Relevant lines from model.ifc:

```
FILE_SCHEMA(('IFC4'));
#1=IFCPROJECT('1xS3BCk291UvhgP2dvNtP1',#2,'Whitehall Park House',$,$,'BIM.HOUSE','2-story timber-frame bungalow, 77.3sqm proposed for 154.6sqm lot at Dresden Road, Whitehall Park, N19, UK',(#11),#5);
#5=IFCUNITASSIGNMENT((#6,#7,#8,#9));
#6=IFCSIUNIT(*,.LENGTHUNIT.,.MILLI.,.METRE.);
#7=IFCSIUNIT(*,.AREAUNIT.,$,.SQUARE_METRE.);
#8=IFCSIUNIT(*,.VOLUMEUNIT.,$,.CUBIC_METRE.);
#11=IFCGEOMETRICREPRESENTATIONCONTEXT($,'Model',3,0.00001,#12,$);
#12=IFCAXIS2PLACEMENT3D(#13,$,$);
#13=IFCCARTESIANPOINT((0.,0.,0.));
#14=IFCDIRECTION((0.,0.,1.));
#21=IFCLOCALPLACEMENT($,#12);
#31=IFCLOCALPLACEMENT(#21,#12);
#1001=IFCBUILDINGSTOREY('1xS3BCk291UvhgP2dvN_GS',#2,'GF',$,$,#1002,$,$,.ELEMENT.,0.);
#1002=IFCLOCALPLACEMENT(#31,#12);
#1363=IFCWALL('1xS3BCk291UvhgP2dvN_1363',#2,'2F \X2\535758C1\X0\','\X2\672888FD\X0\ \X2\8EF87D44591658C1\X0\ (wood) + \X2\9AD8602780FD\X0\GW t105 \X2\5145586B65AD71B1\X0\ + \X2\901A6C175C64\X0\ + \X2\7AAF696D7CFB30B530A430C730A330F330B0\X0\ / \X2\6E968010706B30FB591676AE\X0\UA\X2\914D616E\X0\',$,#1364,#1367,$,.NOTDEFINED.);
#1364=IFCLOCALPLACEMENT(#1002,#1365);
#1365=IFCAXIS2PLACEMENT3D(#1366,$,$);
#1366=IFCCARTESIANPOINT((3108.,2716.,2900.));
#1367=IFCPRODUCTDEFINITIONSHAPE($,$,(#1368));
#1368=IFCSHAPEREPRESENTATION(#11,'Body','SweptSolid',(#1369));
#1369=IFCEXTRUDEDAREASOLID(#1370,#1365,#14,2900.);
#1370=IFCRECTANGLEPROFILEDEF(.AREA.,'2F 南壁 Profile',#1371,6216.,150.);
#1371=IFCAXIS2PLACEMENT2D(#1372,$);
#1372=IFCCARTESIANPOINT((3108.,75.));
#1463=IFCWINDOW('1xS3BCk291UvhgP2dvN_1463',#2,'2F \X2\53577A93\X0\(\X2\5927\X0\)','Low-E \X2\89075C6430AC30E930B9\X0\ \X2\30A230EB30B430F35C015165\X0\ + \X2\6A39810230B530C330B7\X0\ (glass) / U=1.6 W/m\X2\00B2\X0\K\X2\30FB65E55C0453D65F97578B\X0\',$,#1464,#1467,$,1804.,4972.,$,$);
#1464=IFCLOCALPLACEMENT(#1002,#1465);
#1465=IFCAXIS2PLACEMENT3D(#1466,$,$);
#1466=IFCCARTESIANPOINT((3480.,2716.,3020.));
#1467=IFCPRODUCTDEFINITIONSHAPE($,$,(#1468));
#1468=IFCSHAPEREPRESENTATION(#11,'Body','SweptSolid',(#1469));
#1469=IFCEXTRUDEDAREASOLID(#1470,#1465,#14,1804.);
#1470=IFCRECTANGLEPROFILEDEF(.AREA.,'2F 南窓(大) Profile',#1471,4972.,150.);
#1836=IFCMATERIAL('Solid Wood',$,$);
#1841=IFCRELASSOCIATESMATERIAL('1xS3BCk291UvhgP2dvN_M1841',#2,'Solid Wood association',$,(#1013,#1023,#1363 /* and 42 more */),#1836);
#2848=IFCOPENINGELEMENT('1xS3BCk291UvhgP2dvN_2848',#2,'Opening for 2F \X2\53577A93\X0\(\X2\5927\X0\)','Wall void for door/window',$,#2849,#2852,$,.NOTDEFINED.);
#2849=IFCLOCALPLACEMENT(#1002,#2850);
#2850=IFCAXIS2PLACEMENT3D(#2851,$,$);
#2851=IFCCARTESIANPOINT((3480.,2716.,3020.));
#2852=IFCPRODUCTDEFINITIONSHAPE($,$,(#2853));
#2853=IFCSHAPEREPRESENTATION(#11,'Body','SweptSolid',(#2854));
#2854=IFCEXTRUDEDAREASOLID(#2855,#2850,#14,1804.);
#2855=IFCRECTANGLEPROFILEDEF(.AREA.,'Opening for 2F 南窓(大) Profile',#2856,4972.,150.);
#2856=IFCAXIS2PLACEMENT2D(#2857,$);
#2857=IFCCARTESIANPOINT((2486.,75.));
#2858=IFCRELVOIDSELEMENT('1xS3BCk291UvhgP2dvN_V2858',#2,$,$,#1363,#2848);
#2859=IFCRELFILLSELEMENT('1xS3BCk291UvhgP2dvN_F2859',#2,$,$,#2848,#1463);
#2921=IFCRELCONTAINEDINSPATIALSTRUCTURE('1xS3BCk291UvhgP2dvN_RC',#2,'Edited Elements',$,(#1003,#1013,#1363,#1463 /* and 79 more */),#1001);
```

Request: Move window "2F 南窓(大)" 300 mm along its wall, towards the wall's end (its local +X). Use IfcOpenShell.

```python
import ifcopenshell
import ifcopenshell.api.geometry
import ifcopenshell.util.placement
import ifcopenshell.util.unit

model = ifcopenshell.open("model.ifc")
unit_scale = ifcopenshell.util.unit.calculate_unit_scale(model)

window = model.by_guid("1xS3BCk291UvhgP2dvN_1463")
opening = window.FillsVoids[0].RelatingOpeningElement
wall = opening.VoidsElements[0].RelatingBuildingElement

wall_matrix = ifcopenshell.util.placement.get_local_placement(wall.ObjectPlacement)
shift = wall_matrix[:3, 0] * 0.3 / unit_scale
before = ifcopenshell.util.placement.get_local_placement(window.ObjectPlacement)[:3, 3].copy()

# The window is not placed relative to its opening, so move both.
for product in (opening, window):
    matrix = ifcopenshell.util.placement.get_local_placement(product.ObjectPlacement)
    matrix[:3, 3] += shift
    ifcopenshell.api.geometry.edit_object_placement(model, product=product, matrix=matrix, is_si=False)

after = ifcopenshell.util.placement.get_local_placement(window.ObjectPlacement)[:3, 3]
print("window moved by", (after - before).round(3) + 0.0)

model.write("model_edited.ifc")
```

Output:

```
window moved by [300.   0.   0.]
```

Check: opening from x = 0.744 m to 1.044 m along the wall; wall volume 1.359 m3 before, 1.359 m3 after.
